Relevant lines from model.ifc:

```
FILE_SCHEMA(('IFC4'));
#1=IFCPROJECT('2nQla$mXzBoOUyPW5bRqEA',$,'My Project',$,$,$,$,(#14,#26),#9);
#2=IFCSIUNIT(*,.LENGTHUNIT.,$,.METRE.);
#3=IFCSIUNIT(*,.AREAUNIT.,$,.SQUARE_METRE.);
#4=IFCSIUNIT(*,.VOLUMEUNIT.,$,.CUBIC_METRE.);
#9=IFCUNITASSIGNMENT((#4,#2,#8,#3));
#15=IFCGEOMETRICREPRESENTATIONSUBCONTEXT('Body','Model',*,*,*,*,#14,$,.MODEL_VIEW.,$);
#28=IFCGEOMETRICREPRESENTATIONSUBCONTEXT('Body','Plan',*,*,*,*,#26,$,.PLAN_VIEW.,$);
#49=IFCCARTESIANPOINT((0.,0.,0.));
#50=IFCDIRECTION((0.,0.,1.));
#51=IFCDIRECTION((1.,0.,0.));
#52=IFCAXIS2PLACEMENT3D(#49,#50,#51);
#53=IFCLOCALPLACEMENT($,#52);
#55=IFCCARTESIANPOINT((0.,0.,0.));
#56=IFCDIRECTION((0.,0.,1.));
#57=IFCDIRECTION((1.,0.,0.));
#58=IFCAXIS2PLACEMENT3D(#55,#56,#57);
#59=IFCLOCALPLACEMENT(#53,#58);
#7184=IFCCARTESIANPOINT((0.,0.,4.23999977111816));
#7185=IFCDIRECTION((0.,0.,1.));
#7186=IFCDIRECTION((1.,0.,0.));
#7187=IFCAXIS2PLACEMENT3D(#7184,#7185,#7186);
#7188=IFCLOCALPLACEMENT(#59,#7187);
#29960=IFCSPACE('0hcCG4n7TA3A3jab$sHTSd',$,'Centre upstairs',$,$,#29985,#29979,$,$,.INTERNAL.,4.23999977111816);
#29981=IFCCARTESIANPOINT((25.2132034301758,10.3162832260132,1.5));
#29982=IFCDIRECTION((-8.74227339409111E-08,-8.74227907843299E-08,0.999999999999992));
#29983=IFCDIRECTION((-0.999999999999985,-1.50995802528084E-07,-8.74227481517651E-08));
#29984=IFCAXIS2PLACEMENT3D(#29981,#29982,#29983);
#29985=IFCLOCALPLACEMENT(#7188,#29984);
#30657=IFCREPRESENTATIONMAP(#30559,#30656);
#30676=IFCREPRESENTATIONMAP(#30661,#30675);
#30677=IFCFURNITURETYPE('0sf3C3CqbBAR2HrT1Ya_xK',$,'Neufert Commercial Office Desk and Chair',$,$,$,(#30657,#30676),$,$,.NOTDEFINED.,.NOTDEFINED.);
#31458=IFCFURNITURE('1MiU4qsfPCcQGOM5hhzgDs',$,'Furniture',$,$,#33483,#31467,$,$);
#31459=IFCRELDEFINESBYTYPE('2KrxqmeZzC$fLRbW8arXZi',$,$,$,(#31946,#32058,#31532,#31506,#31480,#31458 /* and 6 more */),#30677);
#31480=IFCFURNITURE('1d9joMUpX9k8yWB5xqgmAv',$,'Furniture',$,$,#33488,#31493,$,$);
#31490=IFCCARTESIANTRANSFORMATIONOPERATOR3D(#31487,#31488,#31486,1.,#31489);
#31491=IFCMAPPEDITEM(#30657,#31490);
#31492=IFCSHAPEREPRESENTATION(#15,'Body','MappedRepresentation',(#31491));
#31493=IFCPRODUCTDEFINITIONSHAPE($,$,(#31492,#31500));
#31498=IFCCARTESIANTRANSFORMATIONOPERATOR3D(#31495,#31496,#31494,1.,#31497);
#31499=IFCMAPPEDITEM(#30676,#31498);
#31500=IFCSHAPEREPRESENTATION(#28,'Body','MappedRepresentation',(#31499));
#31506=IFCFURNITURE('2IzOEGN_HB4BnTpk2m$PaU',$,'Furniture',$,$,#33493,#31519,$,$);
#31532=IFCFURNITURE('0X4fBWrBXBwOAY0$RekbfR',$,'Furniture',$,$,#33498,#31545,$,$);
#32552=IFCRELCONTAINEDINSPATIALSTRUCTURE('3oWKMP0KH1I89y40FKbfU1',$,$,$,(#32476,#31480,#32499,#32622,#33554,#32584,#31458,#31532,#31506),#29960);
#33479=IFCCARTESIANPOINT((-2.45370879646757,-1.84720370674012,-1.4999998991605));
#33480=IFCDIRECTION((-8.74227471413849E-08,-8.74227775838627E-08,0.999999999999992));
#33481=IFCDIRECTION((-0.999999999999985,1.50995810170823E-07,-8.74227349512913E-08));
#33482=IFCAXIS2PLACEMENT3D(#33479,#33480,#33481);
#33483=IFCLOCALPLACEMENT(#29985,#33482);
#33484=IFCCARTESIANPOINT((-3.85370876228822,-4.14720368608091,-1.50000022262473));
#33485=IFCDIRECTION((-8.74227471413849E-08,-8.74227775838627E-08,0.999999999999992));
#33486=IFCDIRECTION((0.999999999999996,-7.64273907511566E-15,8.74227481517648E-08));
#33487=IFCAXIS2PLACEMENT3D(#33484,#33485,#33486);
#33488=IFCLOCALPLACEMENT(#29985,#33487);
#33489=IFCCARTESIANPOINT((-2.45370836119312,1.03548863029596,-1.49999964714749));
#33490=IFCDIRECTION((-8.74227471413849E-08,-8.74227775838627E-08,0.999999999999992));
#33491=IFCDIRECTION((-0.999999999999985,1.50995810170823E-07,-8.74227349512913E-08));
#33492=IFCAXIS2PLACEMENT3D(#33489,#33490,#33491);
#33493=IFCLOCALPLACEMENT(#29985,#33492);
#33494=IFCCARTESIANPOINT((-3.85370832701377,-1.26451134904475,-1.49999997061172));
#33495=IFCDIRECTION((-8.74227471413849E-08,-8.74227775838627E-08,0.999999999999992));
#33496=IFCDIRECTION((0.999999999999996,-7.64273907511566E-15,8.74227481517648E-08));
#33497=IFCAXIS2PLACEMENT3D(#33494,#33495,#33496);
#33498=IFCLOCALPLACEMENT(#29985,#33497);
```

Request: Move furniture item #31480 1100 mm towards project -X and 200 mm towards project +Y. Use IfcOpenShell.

```python
import ifcopenshell
import ifcopenshell.api.geometry
import ifcopenshell.util.placement

model = ifcopenshell.open("model.ifc")

item = model.by_id(31480)
matrix = ifcopenshell.util.placement.get_local_placement(item.ObjectPlacement)
matrix[0, 3] -= 1.1
matrix[1, 3] += 0.2
ifcopenshell.api.geometry.edit_object_placement(model, product=item, matrix=matrix, is_si=False)

print(ifcopenshell.util.placement.get_local_placement(item.ObjectPlacement).round(3) + 0.0)

model.write("model-out.ifc")
```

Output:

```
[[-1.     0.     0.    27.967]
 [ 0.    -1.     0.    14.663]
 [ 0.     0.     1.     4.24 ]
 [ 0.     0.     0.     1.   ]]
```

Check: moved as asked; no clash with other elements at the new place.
